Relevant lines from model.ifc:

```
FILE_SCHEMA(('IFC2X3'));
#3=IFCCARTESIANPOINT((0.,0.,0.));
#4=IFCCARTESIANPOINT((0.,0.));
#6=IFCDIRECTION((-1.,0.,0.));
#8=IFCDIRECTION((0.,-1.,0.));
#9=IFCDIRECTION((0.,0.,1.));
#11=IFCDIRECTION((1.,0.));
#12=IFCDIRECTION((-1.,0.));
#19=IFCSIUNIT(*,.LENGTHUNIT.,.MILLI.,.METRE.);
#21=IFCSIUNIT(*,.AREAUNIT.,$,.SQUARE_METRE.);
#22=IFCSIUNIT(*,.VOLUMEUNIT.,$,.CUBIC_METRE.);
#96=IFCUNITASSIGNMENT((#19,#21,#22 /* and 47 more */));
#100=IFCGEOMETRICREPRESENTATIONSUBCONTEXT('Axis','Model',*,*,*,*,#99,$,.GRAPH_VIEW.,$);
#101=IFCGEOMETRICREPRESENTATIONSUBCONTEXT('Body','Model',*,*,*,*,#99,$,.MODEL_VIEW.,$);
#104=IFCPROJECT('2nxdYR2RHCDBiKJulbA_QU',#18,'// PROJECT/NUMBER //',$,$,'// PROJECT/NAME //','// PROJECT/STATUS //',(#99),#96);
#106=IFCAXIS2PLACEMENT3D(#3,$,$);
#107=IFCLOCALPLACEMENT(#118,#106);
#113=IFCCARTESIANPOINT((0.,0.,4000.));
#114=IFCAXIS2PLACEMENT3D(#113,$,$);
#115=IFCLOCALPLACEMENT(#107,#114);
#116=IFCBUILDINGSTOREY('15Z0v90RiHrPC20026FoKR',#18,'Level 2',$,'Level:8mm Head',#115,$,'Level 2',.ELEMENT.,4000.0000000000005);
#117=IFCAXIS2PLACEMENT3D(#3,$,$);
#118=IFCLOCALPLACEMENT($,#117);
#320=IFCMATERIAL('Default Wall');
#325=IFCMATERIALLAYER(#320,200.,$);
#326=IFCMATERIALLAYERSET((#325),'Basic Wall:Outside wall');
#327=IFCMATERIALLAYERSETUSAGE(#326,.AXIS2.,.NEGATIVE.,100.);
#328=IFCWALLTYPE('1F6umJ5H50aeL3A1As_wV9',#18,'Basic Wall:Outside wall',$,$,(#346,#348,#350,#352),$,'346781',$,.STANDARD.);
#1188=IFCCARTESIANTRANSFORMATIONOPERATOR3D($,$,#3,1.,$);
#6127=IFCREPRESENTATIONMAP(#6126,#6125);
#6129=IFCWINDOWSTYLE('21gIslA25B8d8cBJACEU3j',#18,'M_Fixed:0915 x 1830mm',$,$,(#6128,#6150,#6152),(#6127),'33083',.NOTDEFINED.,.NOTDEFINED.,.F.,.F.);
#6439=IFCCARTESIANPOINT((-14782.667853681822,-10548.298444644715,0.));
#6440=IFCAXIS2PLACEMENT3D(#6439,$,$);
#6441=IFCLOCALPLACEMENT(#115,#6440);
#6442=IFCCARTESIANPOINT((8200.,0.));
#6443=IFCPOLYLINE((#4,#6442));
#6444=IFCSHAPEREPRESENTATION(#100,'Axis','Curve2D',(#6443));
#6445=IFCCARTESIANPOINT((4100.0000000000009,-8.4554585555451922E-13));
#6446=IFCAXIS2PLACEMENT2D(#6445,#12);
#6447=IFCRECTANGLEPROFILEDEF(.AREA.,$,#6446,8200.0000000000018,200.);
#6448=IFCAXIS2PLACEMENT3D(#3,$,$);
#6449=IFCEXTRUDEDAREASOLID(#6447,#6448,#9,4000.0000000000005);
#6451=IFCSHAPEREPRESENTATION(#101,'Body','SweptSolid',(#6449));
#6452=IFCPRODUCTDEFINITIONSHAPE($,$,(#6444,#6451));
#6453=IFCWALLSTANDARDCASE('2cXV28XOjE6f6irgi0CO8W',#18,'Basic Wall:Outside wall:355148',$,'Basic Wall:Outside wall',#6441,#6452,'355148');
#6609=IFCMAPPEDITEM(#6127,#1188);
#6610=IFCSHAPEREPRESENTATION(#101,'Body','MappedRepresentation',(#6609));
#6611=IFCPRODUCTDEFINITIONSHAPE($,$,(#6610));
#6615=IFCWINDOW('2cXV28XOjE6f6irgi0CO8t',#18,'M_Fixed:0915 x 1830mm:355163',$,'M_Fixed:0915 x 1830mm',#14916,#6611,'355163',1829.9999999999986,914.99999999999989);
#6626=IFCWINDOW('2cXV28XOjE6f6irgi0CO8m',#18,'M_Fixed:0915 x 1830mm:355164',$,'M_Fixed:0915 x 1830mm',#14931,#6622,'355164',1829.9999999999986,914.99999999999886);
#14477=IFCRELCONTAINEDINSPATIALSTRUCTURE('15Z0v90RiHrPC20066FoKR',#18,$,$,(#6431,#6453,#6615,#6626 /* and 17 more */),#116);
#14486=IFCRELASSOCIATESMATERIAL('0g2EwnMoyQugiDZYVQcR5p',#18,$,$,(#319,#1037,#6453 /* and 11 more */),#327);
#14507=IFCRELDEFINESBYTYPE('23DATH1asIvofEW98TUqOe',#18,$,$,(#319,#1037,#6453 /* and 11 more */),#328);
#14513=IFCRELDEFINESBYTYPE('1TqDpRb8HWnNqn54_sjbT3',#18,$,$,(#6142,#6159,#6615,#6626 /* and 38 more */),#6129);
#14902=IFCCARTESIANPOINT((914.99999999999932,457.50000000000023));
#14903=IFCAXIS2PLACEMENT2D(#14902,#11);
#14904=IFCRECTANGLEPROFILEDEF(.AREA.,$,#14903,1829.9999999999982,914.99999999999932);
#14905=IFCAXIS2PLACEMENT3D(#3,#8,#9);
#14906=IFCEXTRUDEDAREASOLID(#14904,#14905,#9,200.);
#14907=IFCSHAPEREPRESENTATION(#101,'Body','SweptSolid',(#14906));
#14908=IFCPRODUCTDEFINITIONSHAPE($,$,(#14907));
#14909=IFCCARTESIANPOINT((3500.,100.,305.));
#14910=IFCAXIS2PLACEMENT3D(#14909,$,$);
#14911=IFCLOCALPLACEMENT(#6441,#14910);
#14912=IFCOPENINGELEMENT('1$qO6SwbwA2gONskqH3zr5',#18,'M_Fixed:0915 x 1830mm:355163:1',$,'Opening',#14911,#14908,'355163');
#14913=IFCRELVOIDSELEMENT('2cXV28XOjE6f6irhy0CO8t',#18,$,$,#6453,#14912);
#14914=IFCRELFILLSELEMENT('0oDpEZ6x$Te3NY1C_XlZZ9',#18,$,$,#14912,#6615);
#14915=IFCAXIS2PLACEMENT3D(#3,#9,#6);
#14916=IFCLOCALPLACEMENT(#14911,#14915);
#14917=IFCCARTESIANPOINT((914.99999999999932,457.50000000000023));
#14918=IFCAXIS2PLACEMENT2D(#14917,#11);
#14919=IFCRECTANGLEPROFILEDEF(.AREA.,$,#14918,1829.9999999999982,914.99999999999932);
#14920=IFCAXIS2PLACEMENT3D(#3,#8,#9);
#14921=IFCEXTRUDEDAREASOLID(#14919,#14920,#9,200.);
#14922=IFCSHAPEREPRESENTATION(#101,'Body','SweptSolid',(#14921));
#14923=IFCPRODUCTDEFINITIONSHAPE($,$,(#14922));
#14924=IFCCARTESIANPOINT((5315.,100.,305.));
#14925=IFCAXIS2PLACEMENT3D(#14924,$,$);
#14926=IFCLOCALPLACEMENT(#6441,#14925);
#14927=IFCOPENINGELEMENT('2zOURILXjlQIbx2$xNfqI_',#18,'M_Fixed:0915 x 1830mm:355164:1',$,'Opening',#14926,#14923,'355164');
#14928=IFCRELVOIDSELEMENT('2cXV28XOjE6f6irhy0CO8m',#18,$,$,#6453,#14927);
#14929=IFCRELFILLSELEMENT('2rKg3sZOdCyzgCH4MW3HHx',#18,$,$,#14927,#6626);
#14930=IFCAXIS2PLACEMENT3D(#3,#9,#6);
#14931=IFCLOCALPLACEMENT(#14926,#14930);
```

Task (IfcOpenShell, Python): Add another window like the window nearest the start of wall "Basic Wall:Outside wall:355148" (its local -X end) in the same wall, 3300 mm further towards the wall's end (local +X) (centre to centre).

```python
import ifcopenshell
import ifcopenshell.api.feature
import ifcopenshell.api.geometry
import ifcopenshell.api.root
import ifcopenshell.geom
import ifcopenshell.util.element
import ifcopenshell.util.placement
import ifcopenshell.util.shape

model = ifcopenshell.open("model.ifc")
settings = ifcopenshell.geom.settings()


def volume(element):
    """Net volume in cubic metres, openings subtracted."""
    shape = ifcopenshell.geom.create_shape(settings, element)
    return ifcopenshell.util.shape.get_volume(shape.geometry)


def reuse_history(source, copy):
    """copy_class also copies each property set's owner history, people and application; keep the originals."""
    for rel in copy.IsDefinedBy:
        if rel.is_a("IfcRelDefinesByProperties") and (history := rel.RelatingPropertyDefinition.OwnerHistory):
            rel.RelatingPropertyDefinition.OwnerHistory = source.OwnerHistory
            ifcopenshell.util.element.remove_deep2(model, history)


window = model.by_guid("2cXV28XOjE6f6irgi0CO8t")
opening = window.FillsVoids[0].RelatingOpeningElement
wall = opening.VoidsElements[0].RelatingBuildingElement
before = volume(wall)
shift = ifcopenshell.util.placement.get_local_placement(wall.ObjectPlacement)[:3, 0] * 3300.0

# copy_class copies the void relationship, type, container and properties, but no geometry.
new_opening = ifcopenshell.api.root.copy_class(model, product=opening)
new_opening.Representation = ifcopenshell.util.element.copy_deep(
    model, opening.Representation, exclude=["IfcGeometricRepresentationContext", "IfcRepresentationMap"]
)
new_opening.Name = "M_Fixed:0915 x 1830mm"
new_opening.Tag = None
new_window = ifcopenshell.api.root.copy_class(model, product=window)
new_window.Representation = ifcopenshell.util.element.copy_deep(
    model, window.Representation, exclude=["IfcGeometricRepresentationContext", "IfcRepresentationMap"]
)
new_window.Name = "M_Fixed:0915 x 1830mm"
new_window.Tag = None
reuse_history(window, new_window)
fills = ifcopenshell.api.feature.add_filling(model, opening=new_opening, element=new_window)
fills.OwnerHistory = new_window.OwnerHistory  # required in IFC2X3

for old, new in ((opening, new_opening), (window, new_window)):
    matrix = ifcopenshell.util.placement.get_local_placement(old.ObjectPlacement)
    matrix[:3, 3] += shift
    ifcopenshell.api.geometry.edit_object_placement(model, product=new, matrix=matrix, is_si=False)

after = volume(wall)

print(f"wall volume {before:.3f} -> {after:.3f} m3")

model.write("model-out.ifc")
```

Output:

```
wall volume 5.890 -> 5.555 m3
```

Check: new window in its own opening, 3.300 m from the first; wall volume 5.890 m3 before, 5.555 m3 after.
